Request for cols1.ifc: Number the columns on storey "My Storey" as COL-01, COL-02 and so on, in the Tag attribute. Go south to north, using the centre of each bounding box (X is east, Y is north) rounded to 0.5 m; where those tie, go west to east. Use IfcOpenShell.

First a look at what the model holds.

```python
import ifcopenshell
import ifcopenshell.util.element
import ifcopenshell.util.placement

model = ifcopenshell.open("cols1.ifc")
print(model.schema)
storey = next(s for s in model.by_type("IfcBuildingStorey") if s.Name == "My Storey")
columns = [e for e in ifcopenshell.util.element.get_decomposition(storey) if e.is_a("IfcColumn")]
for e in sorted(columns, key=lambda e: e.id()):
    origin = ifcopenshell.util.placement.get_local_placement(e.ObjectPlacement)[:3, 3]
    print(e.id(), e.Tag, e.Name, origin.round(2) + 0.0, sep=" | ")
```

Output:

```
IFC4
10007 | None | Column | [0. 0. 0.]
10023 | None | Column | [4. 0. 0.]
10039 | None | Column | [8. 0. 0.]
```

```python
import ifcopenshell
import ifcopenshell.geom
import ifcopenshell.util.element
import ifcopenshell.util.shape

model = ifcopenshell.open("cols1.ifc")
settings = ifcopenshell.geom.settings()
settings.set("use-world-coords", True)


def centre(element):
    shape = ifcopenshell.geom.create_shape(settings, element)
    return ifcopenshell.util.shape.get_bbox_centroid(shape.geometry)


storey = next(s for s in model.by_type("IfcBuildingStorey") if s.Name == "My Storey")
columns = [e for e in ifcopenshell.util.element.get_decomposition(storey) if e.is_a("IfcColumn")]

# Insertion points can sit at a corner or the storey origin, so sort by the geometry (in metres).
centres = {e: centre(e) for e in columns}
columns.sort(key=lambda e: (round(centres[e][1] / 0.5), centres[e][0]))

for i, e in enumerate(columns, start=1):
    number = f"COL-{i:02d}"
    e.Tag = number
    print(e.id(), number)

model.write("cols1-out.ifc")
```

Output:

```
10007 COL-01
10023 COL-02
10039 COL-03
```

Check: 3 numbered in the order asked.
